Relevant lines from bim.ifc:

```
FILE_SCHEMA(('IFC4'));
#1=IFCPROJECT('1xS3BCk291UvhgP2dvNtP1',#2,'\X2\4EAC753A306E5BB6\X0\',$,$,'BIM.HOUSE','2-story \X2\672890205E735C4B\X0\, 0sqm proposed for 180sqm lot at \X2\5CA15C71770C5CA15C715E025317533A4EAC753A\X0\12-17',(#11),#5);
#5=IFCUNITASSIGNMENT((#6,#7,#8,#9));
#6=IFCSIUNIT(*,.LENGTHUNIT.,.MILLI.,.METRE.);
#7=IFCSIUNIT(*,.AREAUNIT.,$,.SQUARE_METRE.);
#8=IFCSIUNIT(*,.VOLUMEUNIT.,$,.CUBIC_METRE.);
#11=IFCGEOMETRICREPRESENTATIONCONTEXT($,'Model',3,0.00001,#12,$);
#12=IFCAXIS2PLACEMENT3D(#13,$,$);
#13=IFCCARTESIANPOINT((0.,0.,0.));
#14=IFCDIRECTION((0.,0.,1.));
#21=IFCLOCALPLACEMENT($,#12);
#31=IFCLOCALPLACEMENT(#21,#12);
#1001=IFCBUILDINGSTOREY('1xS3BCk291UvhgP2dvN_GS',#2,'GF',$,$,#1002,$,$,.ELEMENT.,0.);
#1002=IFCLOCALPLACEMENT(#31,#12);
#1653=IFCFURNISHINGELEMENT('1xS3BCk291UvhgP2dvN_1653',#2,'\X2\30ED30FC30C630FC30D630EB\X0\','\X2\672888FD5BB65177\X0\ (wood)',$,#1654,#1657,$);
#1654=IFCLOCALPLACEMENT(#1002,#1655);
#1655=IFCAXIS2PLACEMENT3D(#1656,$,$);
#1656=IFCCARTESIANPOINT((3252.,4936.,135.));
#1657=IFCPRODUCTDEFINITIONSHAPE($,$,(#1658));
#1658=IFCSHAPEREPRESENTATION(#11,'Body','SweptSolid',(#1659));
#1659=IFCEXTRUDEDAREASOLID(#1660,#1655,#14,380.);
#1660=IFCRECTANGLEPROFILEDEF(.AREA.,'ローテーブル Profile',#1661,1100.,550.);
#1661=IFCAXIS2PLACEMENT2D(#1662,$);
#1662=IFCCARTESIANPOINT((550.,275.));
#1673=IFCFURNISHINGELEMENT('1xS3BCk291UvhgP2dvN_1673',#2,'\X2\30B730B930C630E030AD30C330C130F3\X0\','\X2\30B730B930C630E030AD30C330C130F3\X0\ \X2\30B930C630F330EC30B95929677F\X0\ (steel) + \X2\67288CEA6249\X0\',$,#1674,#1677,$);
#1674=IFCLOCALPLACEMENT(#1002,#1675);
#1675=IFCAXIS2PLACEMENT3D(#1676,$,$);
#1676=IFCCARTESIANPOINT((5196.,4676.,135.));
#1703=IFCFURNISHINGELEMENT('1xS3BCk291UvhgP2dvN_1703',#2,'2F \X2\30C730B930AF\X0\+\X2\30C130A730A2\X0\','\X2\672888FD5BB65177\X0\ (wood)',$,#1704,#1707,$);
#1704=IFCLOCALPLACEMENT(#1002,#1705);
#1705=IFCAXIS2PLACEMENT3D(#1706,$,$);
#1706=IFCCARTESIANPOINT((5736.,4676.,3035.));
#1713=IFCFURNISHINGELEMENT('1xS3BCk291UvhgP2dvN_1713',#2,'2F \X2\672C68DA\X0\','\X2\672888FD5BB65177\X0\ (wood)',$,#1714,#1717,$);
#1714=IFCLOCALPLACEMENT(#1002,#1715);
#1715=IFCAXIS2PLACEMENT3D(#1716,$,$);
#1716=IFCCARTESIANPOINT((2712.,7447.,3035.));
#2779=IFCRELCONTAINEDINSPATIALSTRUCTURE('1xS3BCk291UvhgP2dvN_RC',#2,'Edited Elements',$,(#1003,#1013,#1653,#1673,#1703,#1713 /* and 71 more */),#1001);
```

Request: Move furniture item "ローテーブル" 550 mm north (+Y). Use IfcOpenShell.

```python
import ifcopenshell
import ifcopenshell.api.geometry
import ifcopenshell.util.placement

model = ifcopenshell.open("bim.ifc")

item = model.by_guid("1xS3BCk291UvhgP2dvN_1653")
matrix = ifcopenshell.util.placement.get_local_placement(item.ObjectPlacement)
matrix[1, 3] += 550.0
ifcopenshell.api.geometry.edit_object_placement(model, product=item, matrix=matrix, is_si=False)

print(ifcopenshell.util.placement.get_local_placement(item.ObjectPlacement).round(3) + 0.0)

model.write("bim_v2.ifc")
```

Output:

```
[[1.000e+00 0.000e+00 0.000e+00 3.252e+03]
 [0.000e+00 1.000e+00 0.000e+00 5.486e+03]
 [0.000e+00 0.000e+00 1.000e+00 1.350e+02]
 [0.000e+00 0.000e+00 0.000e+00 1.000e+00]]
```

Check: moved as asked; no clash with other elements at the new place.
